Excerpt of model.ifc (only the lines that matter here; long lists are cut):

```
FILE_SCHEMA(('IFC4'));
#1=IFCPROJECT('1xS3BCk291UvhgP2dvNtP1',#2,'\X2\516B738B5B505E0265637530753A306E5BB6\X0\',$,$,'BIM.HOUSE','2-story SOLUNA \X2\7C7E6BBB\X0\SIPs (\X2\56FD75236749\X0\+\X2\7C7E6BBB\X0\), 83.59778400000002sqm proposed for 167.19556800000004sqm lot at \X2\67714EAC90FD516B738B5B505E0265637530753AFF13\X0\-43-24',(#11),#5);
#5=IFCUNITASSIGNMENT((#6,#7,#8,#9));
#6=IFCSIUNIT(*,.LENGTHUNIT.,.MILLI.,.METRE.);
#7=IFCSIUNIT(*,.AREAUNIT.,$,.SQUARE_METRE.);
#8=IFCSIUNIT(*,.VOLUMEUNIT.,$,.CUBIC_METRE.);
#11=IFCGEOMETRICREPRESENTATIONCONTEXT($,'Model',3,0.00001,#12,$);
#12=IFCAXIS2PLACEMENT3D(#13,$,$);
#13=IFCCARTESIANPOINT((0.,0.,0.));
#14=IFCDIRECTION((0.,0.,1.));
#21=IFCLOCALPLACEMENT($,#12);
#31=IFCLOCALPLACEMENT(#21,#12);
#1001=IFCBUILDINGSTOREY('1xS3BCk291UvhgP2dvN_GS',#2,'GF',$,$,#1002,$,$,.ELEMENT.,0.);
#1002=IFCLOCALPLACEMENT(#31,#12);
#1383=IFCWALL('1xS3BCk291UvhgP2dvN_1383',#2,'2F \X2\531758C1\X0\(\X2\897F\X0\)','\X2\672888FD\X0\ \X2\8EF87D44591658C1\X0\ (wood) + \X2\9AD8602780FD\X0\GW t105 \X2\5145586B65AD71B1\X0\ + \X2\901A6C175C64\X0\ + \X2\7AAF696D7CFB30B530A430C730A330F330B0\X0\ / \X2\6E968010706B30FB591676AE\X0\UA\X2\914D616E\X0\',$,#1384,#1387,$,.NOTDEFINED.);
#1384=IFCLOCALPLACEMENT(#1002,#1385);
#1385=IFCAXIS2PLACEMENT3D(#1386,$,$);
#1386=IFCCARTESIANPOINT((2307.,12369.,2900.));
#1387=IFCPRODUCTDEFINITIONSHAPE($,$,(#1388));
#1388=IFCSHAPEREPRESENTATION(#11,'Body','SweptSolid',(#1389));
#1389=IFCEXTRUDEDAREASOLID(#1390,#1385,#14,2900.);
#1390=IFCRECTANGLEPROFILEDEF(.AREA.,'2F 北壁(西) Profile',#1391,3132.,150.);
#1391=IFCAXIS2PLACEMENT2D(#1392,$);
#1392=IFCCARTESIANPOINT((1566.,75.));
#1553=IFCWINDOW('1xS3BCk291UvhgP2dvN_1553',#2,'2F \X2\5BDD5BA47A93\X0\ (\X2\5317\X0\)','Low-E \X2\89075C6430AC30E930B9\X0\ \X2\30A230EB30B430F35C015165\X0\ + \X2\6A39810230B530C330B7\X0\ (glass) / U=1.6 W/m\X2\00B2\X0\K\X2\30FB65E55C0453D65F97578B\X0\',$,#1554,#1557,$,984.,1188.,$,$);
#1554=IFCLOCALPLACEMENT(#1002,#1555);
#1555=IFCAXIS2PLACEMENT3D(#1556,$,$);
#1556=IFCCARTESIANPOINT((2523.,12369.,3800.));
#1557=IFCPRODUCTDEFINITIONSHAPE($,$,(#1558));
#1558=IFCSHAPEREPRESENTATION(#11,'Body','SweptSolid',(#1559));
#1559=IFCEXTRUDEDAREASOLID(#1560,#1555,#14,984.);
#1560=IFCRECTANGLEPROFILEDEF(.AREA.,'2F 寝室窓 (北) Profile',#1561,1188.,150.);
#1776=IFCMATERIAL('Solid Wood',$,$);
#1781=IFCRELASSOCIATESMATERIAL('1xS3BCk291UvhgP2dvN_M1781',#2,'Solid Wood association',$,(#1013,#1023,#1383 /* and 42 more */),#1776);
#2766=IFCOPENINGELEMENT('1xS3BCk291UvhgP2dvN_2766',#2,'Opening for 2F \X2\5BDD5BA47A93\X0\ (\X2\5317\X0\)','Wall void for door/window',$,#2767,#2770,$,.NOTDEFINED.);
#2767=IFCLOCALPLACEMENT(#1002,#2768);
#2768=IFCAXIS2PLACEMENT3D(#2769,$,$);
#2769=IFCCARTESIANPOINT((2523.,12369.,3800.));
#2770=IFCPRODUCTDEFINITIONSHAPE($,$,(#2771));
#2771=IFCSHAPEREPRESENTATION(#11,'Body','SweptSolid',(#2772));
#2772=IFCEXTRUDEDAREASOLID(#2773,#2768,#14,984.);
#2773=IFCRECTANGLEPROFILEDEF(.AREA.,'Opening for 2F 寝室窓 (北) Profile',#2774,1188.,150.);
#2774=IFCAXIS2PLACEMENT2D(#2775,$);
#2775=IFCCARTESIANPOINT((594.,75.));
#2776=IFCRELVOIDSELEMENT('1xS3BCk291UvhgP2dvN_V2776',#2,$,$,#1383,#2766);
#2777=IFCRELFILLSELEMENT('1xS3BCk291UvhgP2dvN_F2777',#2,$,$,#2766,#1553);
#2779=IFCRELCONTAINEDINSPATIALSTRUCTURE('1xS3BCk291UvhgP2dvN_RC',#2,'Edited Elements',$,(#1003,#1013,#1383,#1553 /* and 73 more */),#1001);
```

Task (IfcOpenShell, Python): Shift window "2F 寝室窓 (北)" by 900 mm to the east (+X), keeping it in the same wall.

```python
import ifcopenshell
import ifcopenshell.api.geometry
import ifcopenshell.util.placement

model = ifcopenshell.open("model.ifc")

window = model.by_guid("1xS3BCk291UvhgP2dvN_1553")
opening = window.FillsVoids[0].RelatingOpeningElement
wall = opening.VoidsElements[0].RelatingBuildingElement

wall_matrix = ifcopenshell.util.placement.get_local_placement(wall.ObjectPlacement)
shift = wall_matrix[:3, 0] * 900.0
before = ifcopenshell.util.placement.get_local_placement(window.ObjectPlacement)[:3, 3].copy()

# The window is not placed relative to its opening, so move both.
for product in (opening, window):
    matrix = ifcopenshell.util.placement.get_local_placement(product.ObjectPlacement)
    matrix[:3, 3] += shift
    ifcopenshell.api.geometry.edit_object_placement(model, product=product, matrix=matrix, is_si=False)

after = ifcopenshell.util.placement.get_local_placement(window.ObjectPlacement)[:3, 3]
print("window moved by", (after - before).round(3) + 0.0)

model.write("model_v2.ifc")
```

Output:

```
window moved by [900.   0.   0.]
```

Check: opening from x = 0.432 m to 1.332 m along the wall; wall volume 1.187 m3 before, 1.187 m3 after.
